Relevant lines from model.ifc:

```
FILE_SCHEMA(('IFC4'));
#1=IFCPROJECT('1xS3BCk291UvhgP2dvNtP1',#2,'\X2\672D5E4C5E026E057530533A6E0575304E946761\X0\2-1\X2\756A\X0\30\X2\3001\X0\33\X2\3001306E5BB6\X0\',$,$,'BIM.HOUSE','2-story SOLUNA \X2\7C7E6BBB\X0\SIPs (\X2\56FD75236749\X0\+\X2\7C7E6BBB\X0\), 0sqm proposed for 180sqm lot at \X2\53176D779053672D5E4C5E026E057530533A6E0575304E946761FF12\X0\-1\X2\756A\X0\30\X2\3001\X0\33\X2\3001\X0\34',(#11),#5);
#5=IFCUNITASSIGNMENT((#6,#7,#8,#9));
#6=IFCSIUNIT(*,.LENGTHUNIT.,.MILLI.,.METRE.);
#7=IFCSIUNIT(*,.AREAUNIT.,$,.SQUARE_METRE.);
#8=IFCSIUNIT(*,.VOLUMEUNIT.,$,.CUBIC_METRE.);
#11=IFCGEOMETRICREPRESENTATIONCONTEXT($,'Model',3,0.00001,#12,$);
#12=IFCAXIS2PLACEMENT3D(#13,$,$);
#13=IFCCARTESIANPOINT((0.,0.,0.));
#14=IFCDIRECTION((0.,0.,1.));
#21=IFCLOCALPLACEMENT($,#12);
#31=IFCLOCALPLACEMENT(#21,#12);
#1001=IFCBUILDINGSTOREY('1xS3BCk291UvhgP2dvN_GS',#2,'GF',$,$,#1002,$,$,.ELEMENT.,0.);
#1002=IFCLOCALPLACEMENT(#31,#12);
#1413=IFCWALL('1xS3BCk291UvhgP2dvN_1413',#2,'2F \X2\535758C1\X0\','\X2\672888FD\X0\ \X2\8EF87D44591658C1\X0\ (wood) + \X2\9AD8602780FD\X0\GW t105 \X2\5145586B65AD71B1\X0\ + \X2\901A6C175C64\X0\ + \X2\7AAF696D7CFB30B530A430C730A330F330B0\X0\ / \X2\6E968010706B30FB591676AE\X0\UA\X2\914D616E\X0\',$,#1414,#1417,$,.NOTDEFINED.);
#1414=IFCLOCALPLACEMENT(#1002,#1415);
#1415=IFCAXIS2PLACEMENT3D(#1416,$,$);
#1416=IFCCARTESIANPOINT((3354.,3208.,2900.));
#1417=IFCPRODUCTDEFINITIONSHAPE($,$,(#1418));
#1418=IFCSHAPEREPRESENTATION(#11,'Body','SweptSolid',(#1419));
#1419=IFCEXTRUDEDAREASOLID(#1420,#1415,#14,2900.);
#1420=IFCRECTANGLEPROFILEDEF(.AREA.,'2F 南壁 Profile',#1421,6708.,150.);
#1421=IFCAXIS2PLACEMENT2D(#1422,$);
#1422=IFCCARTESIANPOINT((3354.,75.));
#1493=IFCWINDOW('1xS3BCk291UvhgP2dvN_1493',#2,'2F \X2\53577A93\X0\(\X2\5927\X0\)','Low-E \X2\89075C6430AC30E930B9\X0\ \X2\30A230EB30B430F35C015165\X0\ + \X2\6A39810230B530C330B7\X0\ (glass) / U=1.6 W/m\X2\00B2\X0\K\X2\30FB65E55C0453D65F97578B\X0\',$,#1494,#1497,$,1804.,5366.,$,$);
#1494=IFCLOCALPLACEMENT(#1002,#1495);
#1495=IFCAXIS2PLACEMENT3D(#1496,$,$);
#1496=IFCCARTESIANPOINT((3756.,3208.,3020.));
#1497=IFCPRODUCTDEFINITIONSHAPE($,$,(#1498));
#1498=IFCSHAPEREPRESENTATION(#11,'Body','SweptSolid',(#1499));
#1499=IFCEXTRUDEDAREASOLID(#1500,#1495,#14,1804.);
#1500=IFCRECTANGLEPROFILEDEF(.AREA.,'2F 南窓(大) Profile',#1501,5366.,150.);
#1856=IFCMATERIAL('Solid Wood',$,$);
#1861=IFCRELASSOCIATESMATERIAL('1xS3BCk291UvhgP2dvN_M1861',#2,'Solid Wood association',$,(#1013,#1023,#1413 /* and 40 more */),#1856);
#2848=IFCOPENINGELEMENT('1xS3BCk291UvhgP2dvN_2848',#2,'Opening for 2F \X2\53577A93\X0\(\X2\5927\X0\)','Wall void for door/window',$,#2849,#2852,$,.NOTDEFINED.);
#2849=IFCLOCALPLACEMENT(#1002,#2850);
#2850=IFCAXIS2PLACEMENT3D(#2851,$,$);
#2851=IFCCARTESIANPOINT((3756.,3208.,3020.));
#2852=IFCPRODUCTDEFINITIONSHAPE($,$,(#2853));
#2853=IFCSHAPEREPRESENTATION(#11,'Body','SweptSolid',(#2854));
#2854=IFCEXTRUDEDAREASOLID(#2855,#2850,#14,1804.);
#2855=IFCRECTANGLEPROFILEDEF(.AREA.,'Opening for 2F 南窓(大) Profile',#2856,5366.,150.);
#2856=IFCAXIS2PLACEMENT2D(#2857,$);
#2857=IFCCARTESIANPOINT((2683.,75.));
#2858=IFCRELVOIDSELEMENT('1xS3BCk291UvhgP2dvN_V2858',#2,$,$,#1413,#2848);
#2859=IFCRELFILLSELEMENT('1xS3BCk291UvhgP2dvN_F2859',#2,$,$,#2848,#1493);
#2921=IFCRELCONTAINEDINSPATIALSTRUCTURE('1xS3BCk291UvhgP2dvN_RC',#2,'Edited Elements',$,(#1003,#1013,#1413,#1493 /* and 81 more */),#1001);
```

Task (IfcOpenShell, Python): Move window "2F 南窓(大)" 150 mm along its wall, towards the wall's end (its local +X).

```python
import ifcopenshell
import ifcopenshell.api.geometry
import ifcopenshell.util.placement

model = ifcopenshell.open("model.ifc")

window = model.by_guid("1xS3BCk291UvhgP2dvN_1493")
opening = window.FillsVoids[0].RelatingOpeningElement
wall = opening.VoidsElements[0].RelatingBuildingElement

wall_matrix = ifcopenshell.util.placement.get_local_placement(wall.ObjectPlacement)
shift = wall_matrix[:3, 0] * 150.0
before = ifcopenshell.util.placement.get_local_placement(window.ObjectPlacement)[:3, 3].copy()

# The window is not placed relative to its opening, so move both.
for product in (opening, window):
    matrix = ifcopenshell.util.placement.get_local_placement(product.ObjectPlacement)
    matrix[:3, 3] += shift
    ifcopenshell.api.geometry.edit_object_placement(model, product=product, matrix=matrix, is_si=False)

after = ifcopenshell.util.placement.get_local_placement(window.ObjectPlacement)[:3, 3]
print("window moved by", (after - before).round(3) + 0.0)

model.write("model_rev.ifc")
```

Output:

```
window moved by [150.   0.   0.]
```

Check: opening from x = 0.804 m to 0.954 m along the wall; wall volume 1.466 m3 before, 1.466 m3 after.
